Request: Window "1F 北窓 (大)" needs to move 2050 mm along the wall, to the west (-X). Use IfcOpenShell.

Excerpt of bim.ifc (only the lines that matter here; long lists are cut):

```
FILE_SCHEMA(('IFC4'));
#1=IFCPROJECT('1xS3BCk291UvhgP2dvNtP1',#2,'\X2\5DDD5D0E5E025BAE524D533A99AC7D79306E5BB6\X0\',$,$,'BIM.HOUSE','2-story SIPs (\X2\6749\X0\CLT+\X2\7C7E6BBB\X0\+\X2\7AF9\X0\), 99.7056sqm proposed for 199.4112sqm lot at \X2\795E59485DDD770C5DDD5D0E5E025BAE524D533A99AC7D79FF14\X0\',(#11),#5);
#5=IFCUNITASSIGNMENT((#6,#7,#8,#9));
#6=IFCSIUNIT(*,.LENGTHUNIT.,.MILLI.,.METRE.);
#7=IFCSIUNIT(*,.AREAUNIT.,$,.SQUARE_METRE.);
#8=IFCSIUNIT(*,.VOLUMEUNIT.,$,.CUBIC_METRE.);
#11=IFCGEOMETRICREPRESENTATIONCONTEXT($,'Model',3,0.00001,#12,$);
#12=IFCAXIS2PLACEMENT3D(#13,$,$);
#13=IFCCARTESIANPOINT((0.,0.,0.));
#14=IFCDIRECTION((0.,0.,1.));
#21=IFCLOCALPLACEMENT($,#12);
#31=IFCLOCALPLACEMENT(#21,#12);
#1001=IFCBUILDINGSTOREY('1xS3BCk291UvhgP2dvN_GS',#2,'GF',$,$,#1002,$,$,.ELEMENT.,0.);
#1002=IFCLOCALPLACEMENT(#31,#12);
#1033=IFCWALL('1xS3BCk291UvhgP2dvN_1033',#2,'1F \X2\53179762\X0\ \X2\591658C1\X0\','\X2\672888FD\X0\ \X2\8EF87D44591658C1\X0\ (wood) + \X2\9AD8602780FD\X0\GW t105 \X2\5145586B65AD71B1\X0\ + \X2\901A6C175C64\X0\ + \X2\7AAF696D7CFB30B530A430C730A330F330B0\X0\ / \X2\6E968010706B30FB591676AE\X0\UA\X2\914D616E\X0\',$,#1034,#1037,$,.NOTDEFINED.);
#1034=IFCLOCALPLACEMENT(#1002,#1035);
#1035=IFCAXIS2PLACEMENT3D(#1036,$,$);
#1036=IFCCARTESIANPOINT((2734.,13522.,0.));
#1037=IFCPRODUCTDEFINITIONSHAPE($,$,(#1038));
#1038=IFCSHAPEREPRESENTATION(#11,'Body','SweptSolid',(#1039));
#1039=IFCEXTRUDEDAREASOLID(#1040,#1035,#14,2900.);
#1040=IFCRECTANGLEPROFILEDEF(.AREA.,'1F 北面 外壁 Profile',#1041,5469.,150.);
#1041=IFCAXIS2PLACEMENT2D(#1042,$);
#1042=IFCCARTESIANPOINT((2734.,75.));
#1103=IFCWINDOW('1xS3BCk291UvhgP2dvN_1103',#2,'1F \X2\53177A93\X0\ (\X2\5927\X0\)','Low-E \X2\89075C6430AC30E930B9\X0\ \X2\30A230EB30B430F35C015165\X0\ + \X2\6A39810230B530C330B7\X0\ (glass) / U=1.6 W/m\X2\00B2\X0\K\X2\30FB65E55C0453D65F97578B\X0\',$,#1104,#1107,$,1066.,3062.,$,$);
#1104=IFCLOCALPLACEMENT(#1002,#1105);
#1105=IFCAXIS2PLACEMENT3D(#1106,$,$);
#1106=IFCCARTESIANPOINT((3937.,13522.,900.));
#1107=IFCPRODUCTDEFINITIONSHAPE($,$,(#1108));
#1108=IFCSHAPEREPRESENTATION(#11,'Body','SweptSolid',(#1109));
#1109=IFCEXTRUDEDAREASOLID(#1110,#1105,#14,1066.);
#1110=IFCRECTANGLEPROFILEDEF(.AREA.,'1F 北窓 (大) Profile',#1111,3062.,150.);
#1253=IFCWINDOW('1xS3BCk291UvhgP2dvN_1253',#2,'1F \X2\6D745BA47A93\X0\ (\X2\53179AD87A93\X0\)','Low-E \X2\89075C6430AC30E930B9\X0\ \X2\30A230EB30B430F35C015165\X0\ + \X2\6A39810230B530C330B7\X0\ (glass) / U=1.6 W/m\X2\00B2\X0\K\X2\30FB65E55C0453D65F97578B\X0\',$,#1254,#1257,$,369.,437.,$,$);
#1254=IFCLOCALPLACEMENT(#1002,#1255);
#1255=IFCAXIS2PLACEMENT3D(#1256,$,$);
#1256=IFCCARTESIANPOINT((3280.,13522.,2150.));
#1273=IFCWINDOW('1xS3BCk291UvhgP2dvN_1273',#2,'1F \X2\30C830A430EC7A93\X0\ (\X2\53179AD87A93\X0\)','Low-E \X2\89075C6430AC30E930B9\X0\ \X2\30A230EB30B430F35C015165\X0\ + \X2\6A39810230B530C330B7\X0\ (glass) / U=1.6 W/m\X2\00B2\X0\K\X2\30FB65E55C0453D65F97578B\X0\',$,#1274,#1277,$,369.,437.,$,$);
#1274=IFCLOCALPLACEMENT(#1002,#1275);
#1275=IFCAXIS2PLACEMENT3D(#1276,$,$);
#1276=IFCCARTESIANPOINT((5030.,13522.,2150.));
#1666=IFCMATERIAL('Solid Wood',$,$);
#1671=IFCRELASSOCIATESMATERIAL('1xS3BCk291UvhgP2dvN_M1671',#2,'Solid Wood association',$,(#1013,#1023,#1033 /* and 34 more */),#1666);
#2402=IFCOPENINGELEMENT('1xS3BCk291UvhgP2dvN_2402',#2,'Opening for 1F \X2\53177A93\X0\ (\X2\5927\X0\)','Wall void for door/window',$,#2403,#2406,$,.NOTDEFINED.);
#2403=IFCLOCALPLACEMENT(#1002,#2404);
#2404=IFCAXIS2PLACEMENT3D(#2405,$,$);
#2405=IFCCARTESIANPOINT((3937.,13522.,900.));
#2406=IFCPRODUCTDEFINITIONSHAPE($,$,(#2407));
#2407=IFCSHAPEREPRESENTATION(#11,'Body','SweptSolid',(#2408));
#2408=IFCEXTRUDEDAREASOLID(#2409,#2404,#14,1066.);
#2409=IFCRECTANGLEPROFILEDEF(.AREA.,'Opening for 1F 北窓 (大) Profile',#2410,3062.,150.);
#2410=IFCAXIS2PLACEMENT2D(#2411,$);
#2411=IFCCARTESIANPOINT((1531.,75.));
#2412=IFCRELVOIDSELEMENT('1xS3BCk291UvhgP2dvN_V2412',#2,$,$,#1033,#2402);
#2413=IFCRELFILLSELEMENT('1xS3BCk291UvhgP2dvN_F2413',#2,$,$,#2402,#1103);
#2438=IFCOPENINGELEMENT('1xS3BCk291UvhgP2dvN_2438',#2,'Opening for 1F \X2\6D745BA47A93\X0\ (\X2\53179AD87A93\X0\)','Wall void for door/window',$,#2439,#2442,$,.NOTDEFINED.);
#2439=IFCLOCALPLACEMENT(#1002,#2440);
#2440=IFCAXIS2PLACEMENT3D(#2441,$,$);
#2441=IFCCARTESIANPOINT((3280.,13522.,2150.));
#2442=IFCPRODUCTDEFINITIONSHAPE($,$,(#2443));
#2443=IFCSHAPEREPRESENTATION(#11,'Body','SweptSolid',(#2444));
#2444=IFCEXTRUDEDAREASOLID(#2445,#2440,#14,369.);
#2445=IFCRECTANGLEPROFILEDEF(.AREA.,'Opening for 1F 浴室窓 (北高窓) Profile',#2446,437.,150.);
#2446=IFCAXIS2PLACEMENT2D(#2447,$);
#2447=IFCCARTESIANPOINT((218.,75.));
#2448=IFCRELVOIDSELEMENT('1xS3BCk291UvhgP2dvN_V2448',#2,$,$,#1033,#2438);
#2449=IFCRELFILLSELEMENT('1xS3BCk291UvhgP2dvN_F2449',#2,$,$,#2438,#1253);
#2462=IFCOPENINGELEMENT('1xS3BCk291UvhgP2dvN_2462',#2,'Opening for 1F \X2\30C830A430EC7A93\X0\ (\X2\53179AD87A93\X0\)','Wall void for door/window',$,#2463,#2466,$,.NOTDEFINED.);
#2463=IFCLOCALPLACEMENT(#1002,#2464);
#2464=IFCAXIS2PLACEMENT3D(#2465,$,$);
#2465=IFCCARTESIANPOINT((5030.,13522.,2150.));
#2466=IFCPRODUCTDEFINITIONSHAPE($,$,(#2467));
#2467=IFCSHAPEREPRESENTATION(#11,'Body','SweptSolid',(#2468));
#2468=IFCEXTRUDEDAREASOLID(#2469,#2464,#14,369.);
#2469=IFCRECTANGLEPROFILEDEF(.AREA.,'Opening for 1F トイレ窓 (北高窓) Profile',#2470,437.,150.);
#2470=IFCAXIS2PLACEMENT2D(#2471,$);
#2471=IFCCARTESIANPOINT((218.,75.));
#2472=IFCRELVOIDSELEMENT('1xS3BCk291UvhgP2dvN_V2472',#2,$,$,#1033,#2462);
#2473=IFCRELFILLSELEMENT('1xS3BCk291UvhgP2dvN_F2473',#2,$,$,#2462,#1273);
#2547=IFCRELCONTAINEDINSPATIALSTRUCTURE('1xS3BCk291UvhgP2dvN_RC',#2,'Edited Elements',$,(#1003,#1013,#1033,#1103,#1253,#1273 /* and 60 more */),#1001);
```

```python
import ifcopenshell
import ifcopenshell.api.geometry
import ifcopenshell.util.placement

model = ifcopenshell.open("bim.ifc")

window = model.by_guid("1xS3BCk291UvhgP2dvN_1103")
opening = window.FillsVoids[0].RelatingOpeningElement
wall = opening.VoidsElements[0].RelatingBuildingElement

wall_matrix = ifcopenshell.util.placement.get_local_placement(wall.ObjectPlacement)
shift = wall_matrix[:3, 0] * -2050.0
before = ifcopenshell.util.placement.get_local_placement(window.ObjectPlacement)[:3, 3].copy()

# The window is not placed relative to its opening, so move both.
for product in (opening, window):
    matrix = ifcopenshell.util.placement.get_local_placement(product.ObjectPlacement)
    matrix[:3, 3] += shift
    ifcopenshell.api.geometry.edit_object_placement(model, product=product, matrix=matrix, is_si=False)

after = ifcopenshell.util.placement.get_local_placement(window.ObjectPlacement)[:3, 3]
print("window moved by", (after - before).round(3) + 0.0)

model.write("bim_v2.ifc")
```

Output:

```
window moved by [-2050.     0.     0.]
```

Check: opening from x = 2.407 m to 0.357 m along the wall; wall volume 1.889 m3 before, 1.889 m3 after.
